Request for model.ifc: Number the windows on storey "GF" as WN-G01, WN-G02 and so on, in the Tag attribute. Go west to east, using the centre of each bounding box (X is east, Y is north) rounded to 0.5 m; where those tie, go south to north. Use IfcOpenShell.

First a look at what the model holds.

```python
import ifcopenshell
import ifcopenshell.util.element
import ifcopenshell.util.placement

model = ifcopenshell.open("model.ifc")
print(model.schema)
storey = next(s for s in model.by_type("IfcBuildingStorey") if s.Name == "GF")
windows = [e for e in ifcopenshell.util.element.get_decomposition(storey) if e.is_a("IfcWindow")]
for e in sorted(windows, key=lambda e: e.id()):
    origin = ifcopenshell.util.placement.get_local_placement(e.ObjectPlacement)[:3, 3]
    print(e.id(), e.Tag, e.Name, origin.round(2) + 0.0, sep=" | ")
```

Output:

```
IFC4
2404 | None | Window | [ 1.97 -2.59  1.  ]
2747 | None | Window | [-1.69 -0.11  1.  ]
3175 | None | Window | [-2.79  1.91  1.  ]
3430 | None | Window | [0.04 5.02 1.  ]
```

```python
import ifcopenshell
import ifcopenshell.geom
import ifcopenshell.util.element
import ifcopenshell.util.shape

model = ifcopenshell.open("model.ifc")
settings = ifcopenshell.geom.settings()
settings.set("use-world-coords", True)


def centre(element):
    shape = ifcopenshell.geom.create_shape(settings, element)
    return ifcopenshell.util.shape.get_bbox_centroid(shape.geometry)


storey = next(s for s in model.by_type("IfcBuildingStorey") if s.Name == "GF")
windows = [e for e in ifcopenshell.util.element.get_decomposition(storey) if e.is_a("IfcWindow")]

# Insertion points can sit at a corner or the storey origin, so sort by the geometry (in metres).
centres = {e: centre(e) for e in windows}
windows.sort(key=lambda e: (round(centres[e][0] / 0.5), centres[e][1]))

for i, e in enumerate(windows, start=1):
    number = f"WN-G{i:02d}"
    e.Tag = number
    print(e.id(), number)

model.write("model_edited.ifc")
```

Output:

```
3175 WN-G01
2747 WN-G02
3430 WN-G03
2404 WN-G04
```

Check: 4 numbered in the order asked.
